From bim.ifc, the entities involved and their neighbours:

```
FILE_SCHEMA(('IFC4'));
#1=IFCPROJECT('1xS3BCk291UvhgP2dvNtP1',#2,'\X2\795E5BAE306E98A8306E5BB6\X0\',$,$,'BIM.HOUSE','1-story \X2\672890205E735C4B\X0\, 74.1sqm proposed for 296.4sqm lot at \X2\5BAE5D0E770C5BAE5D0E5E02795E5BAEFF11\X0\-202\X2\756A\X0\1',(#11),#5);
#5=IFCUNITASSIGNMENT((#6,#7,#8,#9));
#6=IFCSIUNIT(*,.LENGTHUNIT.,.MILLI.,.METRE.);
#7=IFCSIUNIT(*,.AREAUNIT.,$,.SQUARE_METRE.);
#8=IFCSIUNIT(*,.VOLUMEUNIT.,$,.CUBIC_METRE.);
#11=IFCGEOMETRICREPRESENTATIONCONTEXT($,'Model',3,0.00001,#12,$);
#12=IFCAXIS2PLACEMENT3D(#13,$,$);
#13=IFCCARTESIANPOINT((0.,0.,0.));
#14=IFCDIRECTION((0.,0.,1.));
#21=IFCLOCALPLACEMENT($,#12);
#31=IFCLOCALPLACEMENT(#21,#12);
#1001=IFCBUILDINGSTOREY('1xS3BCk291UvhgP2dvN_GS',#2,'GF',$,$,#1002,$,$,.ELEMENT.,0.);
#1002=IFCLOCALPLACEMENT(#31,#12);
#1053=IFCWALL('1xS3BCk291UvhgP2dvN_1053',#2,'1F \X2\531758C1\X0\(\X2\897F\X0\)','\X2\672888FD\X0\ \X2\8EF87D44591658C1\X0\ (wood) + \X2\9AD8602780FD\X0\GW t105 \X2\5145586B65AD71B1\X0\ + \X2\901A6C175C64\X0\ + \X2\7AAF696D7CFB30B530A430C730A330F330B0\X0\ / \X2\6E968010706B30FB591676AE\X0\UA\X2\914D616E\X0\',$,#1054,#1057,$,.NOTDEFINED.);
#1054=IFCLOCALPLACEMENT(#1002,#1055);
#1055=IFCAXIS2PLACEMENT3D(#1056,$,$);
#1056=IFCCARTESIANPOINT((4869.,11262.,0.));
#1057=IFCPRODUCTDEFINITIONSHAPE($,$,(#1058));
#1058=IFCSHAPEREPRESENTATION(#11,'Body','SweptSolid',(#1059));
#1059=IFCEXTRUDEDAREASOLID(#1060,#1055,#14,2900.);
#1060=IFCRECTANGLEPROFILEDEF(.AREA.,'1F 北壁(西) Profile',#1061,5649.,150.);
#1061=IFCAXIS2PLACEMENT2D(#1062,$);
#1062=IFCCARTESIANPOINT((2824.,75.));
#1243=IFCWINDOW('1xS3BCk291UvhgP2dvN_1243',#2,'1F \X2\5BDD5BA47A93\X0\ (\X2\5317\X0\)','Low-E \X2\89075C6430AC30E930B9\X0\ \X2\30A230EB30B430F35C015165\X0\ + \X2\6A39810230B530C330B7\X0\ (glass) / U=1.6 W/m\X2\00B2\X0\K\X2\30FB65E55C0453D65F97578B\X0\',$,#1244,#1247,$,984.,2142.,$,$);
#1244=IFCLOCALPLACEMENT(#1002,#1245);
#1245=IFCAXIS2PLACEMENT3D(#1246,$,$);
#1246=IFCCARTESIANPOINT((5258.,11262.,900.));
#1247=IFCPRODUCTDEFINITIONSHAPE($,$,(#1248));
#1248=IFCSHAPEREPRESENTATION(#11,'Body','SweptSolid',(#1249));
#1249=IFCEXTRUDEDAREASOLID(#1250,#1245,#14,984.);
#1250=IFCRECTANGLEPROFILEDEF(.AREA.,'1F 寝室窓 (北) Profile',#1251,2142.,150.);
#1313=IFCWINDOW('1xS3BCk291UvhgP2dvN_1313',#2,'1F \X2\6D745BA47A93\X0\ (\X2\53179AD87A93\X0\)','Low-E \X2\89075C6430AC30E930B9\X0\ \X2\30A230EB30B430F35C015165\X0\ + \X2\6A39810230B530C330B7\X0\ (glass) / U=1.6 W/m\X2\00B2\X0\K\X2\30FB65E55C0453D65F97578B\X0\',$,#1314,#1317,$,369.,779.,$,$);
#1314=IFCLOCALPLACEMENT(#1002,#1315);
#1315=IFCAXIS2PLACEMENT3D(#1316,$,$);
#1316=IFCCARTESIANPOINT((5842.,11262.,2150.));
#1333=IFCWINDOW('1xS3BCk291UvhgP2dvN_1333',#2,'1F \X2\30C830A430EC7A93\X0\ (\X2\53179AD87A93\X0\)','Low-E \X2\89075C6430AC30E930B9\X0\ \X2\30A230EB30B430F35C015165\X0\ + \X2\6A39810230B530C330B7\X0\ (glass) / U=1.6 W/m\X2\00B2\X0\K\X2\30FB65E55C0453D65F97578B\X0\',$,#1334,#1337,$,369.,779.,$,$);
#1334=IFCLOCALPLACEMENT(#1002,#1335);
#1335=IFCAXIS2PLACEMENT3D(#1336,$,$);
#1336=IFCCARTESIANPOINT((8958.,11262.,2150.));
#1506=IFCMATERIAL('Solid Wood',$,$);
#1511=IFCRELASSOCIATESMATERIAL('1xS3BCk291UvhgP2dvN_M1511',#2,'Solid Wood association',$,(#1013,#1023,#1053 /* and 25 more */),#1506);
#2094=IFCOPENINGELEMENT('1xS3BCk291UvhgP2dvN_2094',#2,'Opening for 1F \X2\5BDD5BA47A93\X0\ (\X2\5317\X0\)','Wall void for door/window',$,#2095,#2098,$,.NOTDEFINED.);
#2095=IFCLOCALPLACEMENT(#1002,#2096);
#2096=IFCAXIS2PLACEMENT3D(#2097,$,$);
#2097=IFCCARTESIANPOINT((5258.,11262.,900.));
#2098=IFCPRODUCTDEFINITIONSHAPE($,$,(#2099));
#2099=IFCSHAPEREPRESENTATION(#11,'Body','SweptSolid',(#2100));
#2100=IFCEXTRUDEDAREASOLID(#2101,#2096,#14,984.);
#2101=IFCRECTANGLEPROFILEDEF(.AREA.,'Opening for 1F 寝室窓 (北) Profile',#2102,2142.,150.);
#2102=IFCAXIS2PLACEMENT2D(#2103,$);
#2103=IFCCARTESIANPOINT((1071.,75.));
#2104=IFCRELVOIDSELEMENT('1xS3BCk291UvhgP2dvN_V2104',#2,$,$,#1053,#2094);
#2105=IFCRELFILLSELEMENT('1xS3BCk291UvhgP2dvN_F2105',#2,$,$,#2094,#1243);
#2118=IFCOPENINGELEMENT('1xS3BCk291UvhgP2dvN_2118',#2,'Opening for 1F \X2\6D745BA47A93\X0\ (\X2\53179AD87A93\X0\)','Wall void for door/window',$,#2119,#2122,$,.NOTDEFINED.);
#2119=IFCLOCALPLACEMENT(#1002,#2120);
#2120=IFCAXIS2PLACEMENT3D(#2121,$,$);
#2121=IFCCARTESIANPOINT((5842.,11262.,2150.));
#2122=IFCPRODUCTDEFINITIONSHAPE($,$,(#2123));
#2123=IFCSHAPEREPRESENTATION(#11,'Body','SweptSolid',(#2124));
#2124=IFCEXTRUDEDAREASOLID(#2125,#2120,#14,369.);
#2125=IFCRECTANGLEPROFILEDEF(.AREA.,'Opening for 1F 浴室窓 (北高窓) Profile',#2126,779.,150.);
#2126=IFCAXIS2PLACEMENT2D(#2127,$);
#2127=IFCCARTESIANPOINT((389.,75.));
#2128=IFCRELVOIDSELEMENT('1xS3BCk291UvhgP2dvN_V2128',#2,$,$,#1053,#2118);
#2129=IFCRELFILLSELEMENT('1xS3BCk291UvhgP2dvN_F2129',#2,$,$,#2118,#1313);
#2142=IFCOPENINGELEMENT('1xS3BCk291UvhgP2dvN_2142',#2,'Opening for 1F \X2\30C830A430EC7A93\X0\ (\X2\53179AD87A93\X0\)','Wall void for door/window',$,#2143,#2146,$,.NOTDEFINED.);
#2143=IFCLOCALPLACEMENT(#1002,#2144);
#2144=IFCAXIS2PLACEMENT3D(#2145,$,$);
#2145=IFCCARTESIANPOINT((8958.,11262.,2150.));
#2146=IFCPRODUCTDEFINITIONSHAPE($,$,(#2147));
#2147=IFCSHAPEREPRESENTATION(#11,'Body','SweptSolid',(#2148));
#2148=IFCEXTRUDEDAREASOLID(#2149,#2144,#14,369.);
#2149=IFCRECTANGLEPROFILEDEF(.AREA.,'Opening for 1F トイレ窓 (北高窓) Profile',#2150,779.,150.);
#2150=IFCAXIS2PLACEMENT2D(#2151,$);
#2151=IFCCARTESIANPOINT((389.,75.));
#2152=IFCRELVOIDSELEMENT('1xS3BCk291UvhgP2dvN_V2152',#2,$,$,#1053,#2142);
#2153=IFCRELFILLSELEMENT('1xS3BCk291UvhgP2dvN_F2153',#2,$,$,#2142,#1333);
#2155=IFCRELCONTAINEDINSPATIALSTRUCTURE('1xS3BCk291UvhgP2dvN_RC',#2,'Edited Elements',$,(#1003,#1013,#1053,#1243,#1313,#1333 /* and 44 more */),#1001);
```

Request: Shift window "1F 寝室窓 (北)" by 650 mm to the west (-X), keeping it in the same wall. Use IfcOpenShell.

```python
import ifcopenshell
import ifcopenshell.api.geometry
import ifcopenshell.util.placement
import ifcopenshell.util.unit

model = ifcopenshell.open("bim.ifc")
unit_scale = ifcopenshell.util.unit.calculate_unit_scale(model)

window = model.by_guid("1xS3BCk291UvhgP2dvN_1243")
opening = window.FillsVoids[0].RelatingOpeningElement
wall = opening.VoidsElements[0].RelatingBuildingElement

wall_matrix = ifcopenshell.util.placement.get_local_placement(wall.ObjectPlacement)
shift = wall_matrix[:3, 0] * -0.65 / unit_scale
before = ifcopenshell.util.placement.get_local_placement(window.ObjectPlacement)[:3, 3].copy()

# The window is not placed relative to its opening, so move both.
for product in (opening, window):
    matrix = ifcopenshell.util.placement.get_local_placement(product.ObjectPlacement)
    matrix[:3, 3] += shift
    ifcopenshell.api.geometry.edit_object_placement(model, product=product, matrix=matrix, is_si=False)

after = ifcopenshell.util.placement.get_local_placement(window.ObjectPlacement)[:3, 3]
print("window moved by", (after - before).round(3) + 0.0)

model.write("bim_updated.ifc")
```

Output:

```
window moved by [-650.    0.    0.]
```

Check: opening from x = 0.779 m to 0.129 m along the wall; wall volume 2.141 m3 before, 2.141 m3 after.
